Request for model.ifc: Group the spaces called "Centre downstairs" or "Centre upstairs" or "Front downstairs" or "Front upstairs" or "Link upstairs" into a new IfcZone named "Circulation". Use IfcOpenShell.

First a look at what the model holds.

```python
import ifcopenshell

model = ifcopenshell.open("model.ifc")
print(model.schema)
seen = {}
for space in model.by_type("IfcSpace"):
    seen[space.Name] = seen.get(space.Name, 0) + 1
for name, count in sorted(seen.items(), key=str):
    print(count, "x", name)
print("zones:", [z.Name for z in model.by_type("IfcZone")][:20])
```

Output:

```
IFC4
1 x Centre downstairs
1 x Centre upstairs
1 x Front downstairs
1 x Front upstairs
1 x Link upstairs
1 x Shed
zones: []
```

```python
import ifcopenshell
import ifcopenshell.api.group
import ifcopenshell.api.root

model = ifcopenshell.open("model.ifc")

names = {"Centre downstairs", "Centre upstairs", "Front downstairs", "Front upstairs", "Link upstairs"}
spaces = [s for s in model.by_type("IfcSpace") if s.Name in names]

zone = ifcopenshell.api.root.create_entity(model, ifc_class="IfcZone", name="Circulation")
ifcopenshell.api.group.assign_group(model, products=spaces, group=zone)
print(len(spaces), "spaces in", zone.Name)

model.write("model_updated.ifc")
```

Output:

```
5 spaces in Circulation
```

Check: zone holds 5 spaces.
